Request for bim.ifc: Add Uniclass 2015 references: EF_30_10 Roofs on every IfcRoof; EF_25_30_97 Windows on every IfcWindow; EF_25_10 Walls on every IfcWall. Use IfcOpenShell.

First a look at what the model holds.

```python
import ifcopenshell

model = ifcopenshell.open("bim.ifc")
print(model.schema)
print("classifications:", [c.Name for c in model.by_type("IfcClassification")])
for ifc_class in ("IfcDoor", "IfcRoof", "IfcStair", "IfcWall", "IfcWindow"):
    print(ifc_class, len(model.by_type(ifc_class)))
```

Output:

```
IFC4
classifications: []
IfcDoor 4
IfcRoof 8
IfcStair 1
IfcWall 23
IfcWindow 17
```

```python
import ifcopenshell
import ifcopenshell.api.classification

model = ifcopenshell.open("bim.ifc")

system = ifcopenshell.api.classification.add_classification(model, classification="Uniclass 2015")

codes = {
    "IfcRoof": ("EF_30_10", "Roofs"),
    "IfcWindow": ("EF_25_30_97", "Windows"),
    "IfcWall": ("EF_25_10", "Walls"),
}
for ifc_class, (code, name) in codes.items():
    products = model.by_type(ifc_class)
    ifcopenshell.api.classification.add_reference(
        model, products=products, classification=system, identification=code, name=name
    )
    print(code, len(products))

model.write("bim_edited.ifc")
```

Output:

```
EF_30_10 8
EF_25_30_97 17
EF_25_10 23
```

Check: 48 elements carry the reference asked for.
